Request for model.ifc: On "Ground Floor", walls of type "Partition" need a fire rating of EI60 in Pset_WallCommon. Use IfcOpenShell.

First a look at what the model holds.

```python
import ifcopenshell
import ifcopenshell.util.element

model = ifcopenshell.open("model.ifc")
print(model.schema)
storey = next(s for s in model.by_type("IfcBuildingStorey") if s.Name == "Ground Floor")
walls = [e for e in ifcopenshell.util.element.get_decomposition(storey) if e.is_a("IfcWall")]
seen = {}
for e in walls:
    element_type = ifcopenshell.util.element.get_type(e)
    key = (element_type.Name if element_type != e and element_type else None, ifcopenshell.util.element.get_pset(e, "Pset_WallCommon", "FireRating"))
    seen[key] = seen.get(key, 0) + 1
for (name, value), count in sorted(seen.items(), key=str):
    print(count, "x", name, "|", value)
```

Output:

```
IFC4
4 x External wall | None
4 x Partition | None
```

```python
import ifcopenshell
import ifcopenshell.api.pset
import ifcopenshell.util.element

model = ifcopenshell.open("model.ifc")

storey = next(s for s in model.by_type("IfcBuildingStorey") if s.Name == "Ground Floor")
walls = [e for e in ifcopenshell.util.element.get_decomposition(storey) if e.is_a("IfcWall")]

count = 0
for e in walls:
    element_type = ifcopenshell.util.element.get_type(e)
    if element_type in (None, e) or element_type.Name != "Partition":
        continue
    # add_pset returns the element's existing set when there is one.
    pset = ifcopenshell.api.pset.add_pset(model, product=e, name="Pset_WallCommon")
    ifcopenshell.api.pset.edit_pset(model, pset=pset, properties={"FireRating": "EI60"})
    count += 1

print(count, "walls updated")

model.write("model_edited.ifc")
```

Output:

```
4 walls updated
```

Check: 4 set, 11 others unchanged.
